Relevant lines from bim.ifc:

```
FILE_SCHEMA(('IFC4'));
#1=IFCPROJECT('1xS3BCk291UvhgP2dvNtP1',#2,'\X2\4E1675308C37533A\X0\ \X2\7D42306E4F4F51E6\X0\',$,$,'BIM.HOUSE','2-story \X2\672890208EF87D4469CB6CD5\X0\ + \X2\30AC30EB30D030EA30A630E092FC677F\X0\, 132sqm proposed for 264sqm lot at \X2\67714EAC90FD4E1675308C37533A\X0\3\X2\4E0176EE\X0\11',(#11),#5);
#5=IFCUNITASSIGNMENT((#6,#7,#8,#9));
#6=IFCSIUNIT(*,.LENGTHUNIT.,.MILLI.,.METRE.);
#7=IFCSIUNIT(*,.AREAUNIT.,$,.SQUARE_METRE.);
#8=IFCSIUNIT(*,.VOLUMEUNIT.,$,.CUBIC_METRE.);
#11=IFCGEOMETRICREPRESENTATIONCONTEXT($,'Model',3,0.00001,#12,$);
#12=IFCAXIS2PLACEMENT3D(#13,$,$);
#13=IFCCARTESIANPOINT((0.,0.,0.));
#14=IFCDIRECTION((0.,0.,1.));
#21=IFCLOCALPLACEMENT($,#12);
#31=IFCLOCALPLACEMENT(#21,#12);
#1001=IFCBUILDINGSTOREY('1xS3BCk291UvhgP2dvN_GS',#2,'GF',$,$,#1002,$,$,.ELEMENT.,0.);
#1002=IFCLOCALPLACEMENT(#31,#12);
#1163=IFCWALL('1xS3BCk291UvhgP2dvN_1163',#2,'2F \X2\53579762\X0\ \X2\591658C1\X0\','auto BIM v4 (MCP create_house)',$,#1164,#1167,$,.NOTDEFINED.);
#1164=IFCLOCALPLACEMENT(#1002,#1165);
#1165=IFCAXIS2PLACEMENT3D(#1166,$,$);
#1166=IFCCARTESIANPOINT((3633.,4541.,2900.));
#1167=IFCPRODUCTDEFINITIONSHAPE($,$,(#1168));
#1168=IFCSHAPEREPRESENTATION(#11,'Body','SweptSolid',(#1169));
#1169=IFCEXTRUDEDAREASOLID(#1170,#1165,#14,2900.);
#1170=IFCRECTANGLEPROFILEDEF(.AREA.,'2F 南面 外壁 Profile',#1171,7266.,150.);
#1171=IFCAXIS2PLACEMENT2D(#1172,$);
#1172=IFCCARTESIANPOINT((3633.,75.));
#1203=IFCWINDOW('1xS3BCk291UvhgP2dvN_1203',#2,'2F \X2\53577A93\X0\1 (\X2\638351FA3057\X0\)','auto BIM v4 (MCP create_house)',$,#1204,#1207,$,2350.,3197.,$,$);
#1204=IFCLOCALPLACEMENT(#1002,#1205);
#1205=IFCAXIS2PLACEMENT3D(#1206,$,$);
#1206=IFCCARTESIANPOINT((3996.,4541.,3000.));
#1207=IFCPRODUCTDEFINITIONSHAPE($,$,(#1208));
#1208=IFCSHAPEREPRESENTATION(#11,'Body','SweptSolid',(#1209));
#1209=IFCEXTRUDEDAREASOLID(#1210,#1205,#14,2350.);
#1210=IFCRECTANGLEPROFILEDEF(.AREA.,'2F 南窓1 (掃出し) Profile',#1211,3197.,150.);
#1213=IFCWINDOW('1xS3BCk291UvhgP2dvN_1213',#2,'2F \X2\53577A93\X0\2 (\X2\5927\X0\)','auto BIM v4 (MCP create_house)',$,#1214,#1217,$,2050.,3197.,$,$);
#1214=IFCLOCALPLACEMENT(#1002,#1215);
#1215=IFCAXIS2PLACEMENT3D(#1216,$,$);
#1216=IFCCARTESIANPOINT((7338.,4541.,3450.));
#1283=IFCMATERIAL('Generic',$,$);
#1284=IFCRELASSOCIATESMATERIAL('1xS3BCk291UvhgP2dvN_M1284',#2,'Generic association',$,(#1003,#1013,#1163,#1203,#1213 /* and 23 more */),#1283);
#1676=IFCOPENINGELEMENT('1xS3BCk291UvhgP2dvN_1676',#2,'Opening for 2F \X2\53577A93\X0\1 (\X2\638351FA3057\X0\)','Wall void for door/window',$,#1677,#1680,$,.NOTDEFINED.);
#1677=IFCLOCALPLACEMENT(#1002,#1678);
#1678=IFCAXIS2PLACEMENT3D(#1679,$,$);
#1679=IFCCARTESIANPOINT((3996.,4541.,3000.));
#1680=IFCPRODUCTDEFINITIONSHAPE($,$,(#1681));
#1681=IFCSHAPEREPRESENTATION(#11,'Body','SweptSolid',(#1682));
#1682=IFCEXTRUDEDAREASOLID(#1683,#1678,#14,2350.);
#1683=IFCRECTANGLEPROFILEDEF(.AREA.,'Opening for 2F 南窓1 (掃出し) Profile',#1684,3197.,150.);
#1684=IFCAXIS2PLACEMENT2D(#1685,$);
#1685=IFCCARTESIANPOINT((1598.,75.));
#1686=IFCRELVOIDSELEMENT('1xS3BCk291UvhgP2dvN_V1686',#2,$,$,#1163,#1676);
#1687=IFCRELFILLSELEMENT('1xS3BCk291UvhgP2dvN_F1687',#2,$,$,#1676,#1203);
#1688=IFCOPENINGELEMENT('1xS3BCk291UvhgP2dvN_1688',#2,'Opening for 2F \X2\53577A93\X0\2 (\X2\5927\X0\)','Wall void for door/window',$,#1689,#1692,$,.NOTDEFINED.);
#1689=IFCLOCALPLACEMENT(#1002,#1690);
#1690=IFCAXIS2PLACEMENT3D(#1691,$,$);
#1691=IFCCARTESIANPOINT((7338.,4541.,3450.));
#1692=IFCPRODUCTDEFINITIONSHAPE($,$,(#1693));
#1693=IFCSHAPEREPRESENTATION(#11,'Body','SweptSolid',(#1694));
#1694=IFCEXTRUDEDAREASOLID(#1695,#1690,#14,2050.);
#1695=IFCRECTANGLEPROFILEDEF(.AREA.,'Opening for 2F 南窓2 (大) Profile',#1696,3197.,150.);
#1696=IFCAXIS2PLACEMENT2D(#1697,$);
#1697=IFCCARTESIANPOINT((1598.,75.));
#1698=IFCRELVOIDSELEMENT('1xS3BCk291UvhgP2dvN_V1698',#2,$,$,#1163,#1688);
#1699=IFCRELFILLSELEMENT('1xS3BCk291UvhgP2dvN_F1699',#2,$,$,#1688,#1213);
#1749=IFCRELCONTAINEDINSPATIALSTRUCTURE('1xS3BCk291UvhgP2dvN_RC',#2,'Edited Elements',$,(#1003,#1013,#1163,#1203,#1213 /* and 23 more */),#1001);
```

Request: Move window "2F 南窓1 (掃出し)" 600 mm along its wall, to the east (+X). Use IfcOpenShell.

```python
import ifcopenshell
import ifcopenshell.api.geometry
import ifcopenshell.util.placement
import ifcopenshell.util.unit

model = ifcopenshell.open("bim.ifc")
unit_scale = ifcopenshell.util.unit.calculate_unit_scale(model)

window = model.by_id(1203)
opening = window.FillsVoids[0].RelatingOpeningElement
wall = opening.VoidsElements[0].RelatingBuildingElement

wall_matrix = ifcopenshell.util.placement.get_local_placement(wall.ObjectPlacement)
shift = wall_matrix[:3, 0] * 0.6 / unit_scale
before = ifcopenshell.util.placement.get_local_placement(window.ObjectPlacement)[:3, 3].copy()

# The window is not placed relative to its opening, so move both.
for product in (opening, window):
    matrix = ifcopenshell.util.placement.get_local_placement(product.ObjectPlacement)
    matrix[:3, 3] += shift
    ifcopenshell.api.geometry.edit_object_placement(model, product=product, matrix=matrix, is_si=False)

after = ifcopenshell.util.placement.get_local_placement(window.ObjectPlacement)[:3, 3]
print("window moved by", (after - before).round(3) + 0.0)

model.write("bim_rev.ifc")
```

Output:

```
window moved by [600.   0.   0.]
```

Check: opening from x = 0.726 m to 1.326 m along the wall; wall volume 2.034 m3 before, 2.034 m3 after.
